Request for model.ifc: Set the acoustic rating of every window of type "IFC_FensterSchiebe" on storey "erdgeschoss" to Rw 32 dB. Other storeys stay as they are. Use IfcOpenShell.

First a look at what the model holds.

```python
import ifcopenshell
import ifcopenshell.util.element

model = ifcopenshell.open("model.ifc")
print(model.schema)
storey = next(s for s in model.by_type("IfcBuildingStorey") if s.Name == "erdgeschoss")
windows = [e for e in ifcopenshell.util.element.get_decomposition(storey) if e.is_a("IfcWindow")]
seen = {}
for e in windows:
    element_type = ifcopenshell.util.element.get_type(e)
    key = (element_type.Name if element_type != e and element_type else None, ifcopenshell.util.element.get_pset(e, "Pset_WindowCommon", "AcousticRating"))
    seen[key] = seen.get(key, 0) + 1
for (name, value), count in sorted(seen.items(), key=str):
    print(count, "x", name, "|", value)
```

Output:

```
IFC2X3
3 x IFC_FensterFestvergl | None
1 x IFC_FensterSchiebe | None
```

```python
import ifcopenshell
import ifcopenshell.api.pset
import ifcopenshell.util.element

model = ifcopenshell.open("model.ifc")

storey = next(s for s in model.by_type("IfcBuildingStorey") if s.Name == "erdgeschoss")
windows = [e for e in ifcopenshell.util.element.get_decomposition(storey) if e.is_a("IfcWindow")]

count = 0
for e in windows:
    element_type = ifcopenshell.util.element.get_type(e)
    if element_type in (None, e) or element_type.Name != "IFC_FensterSchiebe":
        continue
    # add_pset returns the element's existing set when there is one.
    pset = ifcopenshell.api.pset.add_pset(model, product=e, name="Pset_WindowCommon")
    ifcopenshell.api.pset.edit_pset(model, pset=pset, properties={"AcousticRating": "Rw 32 dB"})
    count += 1

print(count, "windows updated")

model.write("model_edited.ifc")
```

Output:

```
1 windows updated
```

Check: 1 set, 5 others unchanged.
